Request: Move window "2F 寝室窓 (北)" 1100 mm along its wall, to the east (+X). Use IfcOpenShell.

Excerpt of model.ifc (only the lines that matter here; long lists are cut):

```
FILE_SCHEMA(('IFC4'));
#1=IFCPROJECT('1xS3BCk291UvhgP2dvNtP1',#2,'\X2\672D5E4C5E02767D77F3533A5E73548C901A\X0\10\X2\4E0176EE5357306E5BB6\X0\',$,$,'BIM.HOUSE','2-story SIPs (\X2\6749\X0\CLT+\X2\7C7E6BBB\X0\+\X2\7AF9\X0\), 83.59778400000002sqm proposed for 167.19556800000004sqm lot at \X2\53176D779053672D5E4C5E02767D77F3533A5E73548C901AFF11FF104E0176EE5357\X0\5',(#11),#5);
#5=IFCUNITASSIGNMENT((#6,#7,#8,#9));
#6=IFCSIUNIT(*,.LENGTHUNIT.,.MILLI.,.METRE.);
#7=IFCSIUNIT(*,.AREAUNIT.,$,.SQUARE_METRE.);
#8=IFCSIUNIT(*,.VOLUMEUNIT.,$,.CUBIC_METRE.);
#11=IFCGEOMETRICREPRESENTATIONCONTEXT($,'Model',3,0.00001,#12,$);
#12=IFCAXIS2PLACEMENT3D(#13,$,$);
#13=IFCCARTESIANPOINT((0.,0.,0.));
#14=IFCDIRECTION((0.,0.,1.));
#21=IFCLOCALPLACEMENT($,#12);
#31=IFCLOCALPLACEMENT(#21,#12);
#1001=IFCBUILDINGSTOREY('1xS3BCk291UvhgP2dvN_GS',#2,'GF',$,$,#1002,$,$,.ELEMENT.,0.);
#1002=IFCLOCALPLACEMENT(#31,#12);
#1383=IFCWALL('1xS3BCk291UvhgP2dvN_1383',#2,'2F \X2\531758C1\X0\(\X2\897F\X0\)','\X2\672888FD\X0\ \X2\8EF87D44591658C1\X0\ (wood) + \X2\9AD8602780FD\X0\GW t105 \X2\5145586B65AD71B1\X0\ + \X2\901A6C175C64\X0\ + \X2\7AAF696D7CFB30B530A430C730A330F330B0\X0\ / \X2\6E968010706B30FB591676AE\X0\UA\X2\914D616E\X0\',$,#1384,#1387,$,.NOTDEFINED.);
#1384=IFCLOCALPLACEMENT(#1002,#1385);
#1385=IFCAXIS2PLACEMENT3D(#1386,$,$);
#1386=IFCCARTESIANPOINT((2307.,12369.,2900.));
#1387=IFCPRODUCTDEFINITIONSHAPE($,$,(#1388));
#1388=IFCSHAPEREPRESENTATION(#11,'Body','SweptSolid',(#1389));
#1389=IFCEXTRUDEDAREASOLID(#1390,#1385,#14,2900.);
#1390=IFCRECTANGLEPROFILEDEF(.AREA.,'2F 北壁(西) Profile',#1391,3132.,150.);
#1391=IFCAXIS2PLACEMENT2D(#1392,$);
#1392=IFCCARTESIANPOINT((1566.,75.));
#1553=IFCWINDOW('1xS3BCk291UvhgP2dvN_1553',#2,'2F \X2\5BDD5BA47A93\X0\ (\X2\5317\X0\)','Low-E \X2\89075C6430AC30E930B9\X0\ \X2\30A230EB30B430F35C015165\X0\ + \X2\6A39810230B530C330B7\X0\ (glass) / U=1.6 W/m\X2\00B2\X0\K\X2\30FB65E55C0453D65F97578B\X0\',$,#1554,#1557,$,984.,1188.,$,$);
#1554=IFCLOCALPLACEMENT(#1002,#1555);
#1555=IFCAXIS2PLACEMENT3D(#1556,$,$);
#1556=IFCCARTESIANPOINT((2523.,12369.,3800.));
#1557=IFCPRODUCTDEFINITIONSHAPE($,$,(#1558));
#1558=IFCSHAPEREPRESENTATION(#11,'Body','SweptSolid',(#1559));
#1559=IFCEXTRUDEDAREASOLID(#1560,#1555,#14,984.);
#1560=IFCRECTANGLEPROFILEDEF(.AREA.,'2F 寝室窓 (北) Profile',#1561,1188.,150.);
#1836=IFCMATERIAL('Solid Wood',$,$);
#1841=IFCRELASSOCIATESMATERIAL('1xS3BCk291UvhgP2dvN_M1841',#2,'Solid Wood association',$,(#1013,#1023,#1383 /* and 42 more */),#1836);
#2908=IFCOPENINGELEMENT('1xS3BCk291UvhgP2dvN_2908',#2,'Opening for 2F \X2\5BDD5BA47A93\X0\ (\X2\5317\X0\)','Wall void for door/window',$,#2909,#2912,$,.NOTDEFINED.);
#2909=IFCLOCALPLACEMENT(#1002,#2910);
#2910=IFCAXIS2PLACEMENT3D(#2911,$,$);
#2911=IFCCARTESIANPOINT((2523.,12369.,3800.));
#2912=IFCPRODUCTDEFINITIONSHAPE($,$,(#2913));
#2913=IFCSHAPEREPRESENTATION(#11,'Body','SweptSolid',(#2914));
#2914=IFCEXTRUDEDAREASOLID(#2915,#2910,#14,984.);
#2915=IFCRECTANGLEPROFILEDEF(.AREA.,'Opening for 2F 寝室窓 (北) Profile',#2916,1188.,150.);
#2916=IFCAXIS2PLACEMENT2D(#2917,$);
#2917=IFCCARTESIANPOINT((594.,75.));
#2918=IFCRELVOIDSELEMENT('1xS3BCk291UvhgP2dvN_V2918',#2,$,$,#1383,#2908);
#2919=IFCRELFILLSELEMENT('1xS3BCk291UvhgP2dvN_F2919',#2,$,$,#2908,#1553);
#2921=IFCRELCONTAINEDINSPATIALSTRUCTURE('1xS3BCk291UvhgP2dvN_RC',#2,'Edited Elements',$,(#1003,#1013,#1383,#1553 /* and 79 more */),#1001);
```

```python
import ifcopenshell
import ifcopenshell.api.geometry
import ifcopenshell.util.placement

model = ifcopenshell.open("model.ifc")

window = model.by_guid("1xS3BCk291UvhgP2dvN_1553")
opening = window.FillsVoids[0].RelatingOpeningElement
wall = opening.VoidsElements[0].RelatingBuildingElement

wall_matrix = ifcopenshell.util.placement.get_local_placement(wall.ObjectPlacement)
shift = wall_matrix[:3, 0] * 1100.0
before = ifcopenshell.util.placement.get_local_placement(window.ObjectPlacement)[:3, 3].copy()

# The window is not placed relative to its opening, so move both.
for product in (opening, window):
    matrix = ifcopenshell.util.placement.get_local_placement(product.ObjectPlacement)
    matrix[:3, 3] += shift
    ifcopenshell.api.geometry.edit_object_placement(model, product=product, matrix=matrix, is_si=False)

after = ifcopenshell.util.placement.get_local_placement(window.ObjectPlacement)[:3, 3]
print("window moved by", (after - before).round(3) + 0.0)

model.write("model_updated.ifc")
```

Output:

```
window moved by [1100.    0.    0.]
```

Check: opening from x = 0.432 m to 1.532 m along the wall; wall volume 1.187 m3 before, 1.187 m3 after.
